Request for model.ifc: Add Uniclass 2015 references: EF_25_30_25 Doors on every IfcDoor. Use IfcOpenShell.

First a look at what the model holds.

```python
import ifcopenshell

model = ifcopenshell.open("model.ifc")
print(model.schema)
print("classifications:", [c.Name for c in model.by_type("IfcClassification")])
for ifc_class in ("IfcDoor", "IfcRoof", "IfcStair", "IfcWall", "IfcWindow"):
    print(ifc_class, len(model.by_type(ifc_class)))
```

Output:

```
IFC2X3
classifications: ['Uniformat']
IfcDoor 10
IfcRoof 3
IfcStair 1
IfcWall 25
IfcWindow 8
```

```python
import ifcopenshell
import ifcopenshell.api.classification

model = ifcopenshell.open("model.ifc")

# IFC2X3 requires Source and Edition and has no link from the project to the system.
system = model.create_entity("IfcClassification", Source="NBS", Edition="2015", Name="Uniclass 2015")

codes = {
    "IfcDoor": ("EF_25_30_25", "Doors"),
}
for ifc_class, (code, name) in codes.items():
    products = model.by_type(ifc_class)
    ifcopenshell.api.classification.add_reference(
        model, products=products, classification=system, identification=code, name=name
    )
    print(code, len(products))

model.write("model_v2.ifc")
```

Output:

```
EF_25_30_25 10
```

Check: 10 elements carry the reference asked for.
